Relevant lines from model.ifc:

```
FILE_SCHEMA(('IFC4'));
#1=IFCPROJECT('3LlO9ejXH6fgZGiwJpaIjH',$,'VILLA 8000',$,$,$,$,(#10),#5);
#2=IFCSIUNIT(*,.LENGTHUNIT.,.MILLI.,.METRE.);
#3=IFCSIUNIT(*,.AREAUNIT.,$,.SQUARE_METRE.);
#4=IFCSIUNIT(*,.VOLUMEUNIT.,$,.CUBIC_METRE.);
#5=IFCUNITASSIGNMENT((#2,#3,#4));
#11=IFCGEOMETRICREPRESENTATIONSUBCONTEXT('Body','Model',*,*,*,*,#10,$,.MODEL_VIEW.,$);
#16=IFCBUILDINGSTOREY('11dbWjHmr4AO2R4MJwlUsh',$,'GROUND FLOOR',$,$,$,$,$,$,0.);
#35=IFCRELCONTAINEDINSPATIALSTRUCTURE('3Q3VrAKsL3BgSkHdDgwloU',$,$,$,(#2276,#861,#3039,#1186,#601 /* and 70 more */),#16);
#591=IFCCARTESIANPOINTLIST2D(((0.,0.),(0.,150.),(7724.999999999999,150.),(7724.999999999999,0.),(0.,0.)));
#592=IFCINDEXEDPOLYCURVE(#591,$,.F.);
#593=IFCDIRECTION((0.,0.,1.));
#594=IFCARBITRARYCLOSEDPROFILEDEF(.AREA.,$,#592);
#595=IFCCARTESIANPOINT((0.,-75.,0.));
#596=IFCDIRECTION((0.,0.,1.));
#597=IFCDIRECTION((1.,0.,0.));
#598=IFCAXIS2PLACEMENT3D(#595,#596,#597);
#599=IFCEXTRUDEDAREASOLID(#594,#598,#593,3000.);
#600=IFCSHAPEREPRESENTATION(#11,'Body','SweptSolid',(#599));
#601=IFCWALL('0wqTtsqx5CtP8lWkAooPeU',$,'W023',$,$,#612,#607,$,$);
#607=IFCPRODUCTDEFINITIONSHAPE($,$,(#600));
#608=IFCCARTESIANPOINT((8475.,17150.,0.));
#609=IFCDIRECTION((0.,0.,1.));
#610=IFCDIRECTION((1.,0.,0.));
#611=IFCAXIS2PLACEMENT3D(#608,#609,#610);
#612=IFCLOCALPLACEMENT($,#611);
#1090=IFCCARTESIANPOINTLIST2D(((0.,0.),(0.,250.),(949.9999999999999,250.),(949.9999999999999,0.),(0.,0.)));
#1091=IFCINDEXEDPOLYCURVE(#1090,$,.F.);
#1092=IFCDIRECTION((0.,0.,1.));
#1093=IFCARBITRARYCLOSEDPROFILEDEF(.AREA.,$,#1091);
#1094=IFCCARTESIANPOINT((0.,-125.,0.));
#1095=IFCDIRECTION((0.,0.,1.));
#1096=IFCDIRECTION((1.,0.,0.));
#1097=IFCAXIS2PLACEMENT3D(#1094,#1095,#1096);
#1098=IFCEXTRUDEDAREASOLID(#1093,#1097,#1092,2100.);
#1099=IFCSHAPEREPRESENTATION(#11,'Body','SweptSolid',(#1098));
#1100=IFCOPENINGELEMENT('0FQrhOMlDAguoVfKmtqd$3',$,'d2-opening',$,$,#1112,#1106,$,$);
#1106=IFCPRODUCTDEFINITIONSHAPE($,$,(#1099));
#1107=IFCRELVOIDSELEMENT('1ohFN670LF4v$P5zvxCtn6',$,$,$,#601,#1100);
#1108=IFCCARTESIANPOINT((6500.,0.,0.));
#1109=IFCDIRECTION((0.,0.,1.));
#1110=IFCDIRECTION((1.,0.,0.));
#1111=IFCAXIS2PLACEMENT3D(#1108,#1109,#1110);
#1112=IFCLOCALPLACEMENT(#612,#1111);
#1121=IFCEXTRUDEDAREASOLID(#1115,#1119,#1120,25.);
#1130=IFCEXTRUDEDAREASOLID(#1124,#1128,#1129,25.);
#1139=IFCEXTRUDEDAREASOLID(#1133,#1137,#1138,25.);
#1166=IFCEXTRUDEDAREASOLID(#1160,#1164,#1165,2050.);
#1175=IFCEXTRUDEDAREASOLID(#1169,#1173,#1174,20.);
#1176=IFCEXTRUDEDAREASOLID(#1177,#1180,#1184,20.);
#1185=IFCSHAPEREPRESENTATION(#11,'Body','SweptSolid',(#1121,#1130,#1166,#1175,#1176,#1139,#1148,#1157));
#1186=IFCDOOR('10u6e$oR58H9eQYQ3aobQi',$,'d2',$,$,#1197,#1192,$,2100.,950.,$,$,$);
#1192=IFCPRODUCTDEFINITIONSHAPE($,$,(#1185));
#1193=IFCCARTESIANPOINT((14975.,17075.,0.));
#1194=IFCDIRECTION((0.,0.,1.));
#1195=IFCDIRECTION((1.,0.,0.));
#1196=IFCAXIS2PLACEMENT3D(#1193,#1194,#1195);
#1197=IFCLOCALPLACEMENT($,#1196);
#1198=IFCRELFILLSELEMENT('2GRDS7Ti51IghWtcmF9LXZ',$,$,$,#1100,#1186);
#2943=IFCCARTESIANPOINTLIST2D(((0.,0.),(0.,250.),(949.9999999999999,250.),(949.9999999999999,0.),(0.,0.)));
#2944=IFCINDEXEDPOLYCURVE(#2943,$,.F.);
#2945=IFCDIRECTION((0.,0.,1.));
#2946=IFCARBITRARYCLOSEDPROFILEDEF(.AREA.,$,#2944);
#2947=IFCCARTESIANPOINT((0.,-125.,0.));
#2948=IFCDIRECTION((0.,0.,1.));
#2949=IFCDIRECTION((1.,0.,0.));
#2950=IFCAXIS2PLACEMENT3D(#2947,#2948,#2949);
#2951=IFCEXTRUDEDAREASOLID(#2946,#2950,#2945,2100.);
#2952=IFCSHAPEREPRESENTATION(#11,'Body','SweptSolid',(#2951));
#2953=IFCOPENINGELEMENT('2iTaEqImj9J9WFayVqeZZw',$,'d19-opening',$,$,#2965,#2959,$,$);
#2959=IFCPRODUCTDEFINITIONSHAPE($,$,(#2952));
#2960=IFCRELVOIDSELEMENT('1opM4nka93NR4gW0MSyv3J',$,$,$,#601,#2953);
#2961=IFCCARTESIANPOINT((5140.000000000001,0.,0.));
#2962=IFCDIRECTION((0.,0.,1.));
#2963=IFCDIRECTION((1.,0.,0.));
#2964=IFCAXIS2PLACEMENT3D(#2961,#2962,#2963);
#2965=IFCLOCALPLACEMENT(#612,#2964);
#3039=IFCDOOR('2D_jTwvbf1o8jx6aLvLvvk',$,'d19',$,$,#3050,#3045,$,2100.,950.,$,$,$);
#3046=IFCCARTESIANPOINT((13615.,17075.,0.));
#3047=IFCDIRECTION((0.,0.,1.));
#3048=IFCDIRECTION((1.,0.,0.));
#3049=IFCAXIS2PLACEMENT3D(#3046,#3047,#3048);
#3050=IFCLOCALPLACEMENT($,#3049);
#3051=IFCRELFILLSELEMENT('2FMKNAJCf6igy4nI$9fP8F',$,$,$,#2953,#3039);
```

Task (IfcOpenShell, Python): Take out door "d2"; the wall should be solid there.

```python
import ifcopenshell
import ifcopenshell.api.feature
import ifcopenshell.api.root
import ifcopenshell.geom
import ifcopenshell.util.shape

model = ifcopenshell.open("model.ifc")
settings = ifcopenshell.geom.settings()


def volume(element):
    """Net volume in cubic metres, openings subtracted."""
    shape = ifcopenshell.geom.create_shape(settings, element)
    return ifcopenshell.util.shape.get_volume(shape.geometry)


door = model.by_guid("10u6e$oR58H9eQYQ3aobQi")
opening = door.FillsVoids[0].RelatingOpeningElement
wall = opening.VoidsElements[0].RelatingBuildingElement
before = volume(wall)

ifcopenshell.api.root.remove_product(model, product=door)
ifcopenshell.api.feature.remove_feature(model, feature=opening)

after = volume(wall)

print(f"wall volume {before:.3f} -> {after:.3f} m3")

model.write("model_edited.ifc")
```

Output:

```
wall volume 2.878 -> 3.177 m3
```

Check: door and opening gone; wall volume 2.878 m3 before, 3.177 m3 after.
